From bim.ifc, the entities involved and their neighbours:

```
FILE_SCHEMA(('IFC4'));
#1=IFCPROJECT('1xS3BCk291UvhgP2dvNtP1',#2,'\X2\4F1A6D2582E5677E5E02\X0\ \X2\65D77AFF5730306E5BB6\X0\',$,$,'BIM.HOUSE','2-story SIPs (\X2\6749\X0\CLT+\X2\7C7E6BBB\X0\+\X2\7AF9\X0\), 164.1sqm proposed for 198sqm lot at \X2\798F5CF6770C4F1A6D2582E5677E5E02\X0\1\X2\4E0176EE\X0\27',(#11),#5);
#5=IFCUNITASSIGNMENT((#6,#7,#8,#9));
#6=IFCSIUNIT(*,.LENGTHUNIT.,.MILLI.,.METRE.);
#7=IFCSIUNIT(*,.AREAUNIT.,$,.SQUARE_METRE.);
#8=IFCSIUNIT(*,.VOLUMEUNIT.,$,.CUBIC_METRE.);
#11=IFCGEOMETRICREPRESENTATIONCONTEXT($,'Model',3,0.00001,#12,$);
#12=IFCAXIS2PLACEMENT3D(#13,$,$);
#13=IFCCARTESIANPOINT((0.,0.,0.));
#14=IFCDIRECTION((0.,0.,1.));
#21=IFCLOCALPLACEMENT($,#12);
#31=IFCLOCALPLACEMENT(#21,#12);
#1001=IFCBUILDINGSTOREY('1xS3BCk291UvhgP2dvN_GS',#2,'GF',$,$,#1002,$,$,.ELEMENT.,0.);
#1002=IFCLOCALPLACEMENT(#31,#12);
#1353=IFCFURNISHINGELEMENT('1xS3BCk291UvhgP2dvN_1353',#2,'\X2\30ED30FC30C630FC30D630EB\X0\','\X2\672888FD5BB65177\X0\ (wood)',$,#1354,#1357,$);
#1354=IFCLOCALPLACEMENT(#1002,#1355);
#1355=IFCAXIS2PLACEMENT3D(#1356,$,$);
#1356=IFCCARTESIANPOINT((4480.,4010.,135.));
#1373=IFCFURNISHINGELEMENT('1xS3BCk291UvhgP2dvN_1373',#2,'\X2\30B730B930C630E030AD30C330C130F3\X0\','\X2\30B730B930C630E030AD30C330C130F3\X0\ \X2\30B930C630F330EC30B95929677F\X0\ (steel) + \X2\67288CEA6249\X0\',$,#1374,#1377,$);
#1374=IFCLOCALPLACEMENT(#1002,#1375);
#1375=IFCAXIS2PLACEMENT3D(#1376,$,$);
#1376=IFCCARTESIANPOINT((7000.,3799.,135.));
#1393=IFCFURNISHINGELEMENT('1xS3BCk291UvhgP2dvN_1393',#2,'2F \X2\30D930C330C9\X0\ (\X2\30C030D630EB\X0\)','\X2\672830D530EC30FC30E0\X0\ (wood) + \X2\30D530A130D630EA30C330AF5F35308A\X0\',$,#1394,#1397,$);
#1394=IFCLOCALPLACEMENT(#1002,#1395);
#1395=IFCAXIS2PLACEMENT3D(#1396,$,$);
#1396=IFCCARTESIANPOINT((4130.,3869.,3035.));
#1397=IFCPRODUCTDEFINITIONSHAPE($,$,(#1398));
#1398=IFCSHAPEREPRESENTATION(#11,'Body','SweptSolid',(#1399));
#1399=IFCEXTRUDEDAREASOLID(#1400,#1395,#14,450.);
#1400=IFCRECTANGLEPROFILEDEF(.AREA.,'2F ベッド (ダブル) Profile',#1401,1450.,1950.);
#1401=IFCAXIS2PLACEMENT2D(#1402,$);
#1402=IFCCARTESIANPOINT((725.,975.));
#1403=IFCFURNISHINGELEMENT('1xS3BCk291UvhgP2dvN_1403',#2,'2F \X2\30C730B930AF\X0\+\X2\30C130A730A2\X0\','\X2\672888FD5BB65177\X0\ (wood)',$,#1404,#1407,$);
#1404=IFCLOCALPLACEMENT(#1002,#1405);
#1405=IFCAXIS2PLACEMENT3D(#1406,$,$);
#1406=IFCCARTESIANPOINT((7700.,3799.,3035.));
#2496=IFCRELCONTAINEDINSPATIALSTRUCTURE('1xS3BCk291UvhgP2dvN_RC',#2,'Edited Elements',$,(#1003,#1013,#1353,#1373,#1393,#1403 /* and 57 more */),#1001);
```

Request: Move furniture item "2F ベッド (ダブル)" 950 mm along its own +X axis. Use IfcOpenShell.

```python
import ifcopenshell
import ifcopenshell.api.geometry
import ifcopenshell.util.placement
import ifcopenshell.util.unit

model = ifcopenshell.open("bim.ifc")
unit_scale = ifcopenshell.util.unit.calculate_unit_scale(model)

item = model.by_id(1393)
matrix = ifcopenshell.util.placement.get_local_placement(item.ObjectPlacement)
matrix[:3, 3] += matrix[:3, 0] * 0.95 / unit_scale
ifcopenshell.api.geometry.edit_object_placement(model, product=item, matrix=matrix, is_si=False)

print(ifcopenshell.util.placement.get_local_placement(item.ObjectPlacement).round(3) + 0.0)

model.write("bim_updated.ifc")
```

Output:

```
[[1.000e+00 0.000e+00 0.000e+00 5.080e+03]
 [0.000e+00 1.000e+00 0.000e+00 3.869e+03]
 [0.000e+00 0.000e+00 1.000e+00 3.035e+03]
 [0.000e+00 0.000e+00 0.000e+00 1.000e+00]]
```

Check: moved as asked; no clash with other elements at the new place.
